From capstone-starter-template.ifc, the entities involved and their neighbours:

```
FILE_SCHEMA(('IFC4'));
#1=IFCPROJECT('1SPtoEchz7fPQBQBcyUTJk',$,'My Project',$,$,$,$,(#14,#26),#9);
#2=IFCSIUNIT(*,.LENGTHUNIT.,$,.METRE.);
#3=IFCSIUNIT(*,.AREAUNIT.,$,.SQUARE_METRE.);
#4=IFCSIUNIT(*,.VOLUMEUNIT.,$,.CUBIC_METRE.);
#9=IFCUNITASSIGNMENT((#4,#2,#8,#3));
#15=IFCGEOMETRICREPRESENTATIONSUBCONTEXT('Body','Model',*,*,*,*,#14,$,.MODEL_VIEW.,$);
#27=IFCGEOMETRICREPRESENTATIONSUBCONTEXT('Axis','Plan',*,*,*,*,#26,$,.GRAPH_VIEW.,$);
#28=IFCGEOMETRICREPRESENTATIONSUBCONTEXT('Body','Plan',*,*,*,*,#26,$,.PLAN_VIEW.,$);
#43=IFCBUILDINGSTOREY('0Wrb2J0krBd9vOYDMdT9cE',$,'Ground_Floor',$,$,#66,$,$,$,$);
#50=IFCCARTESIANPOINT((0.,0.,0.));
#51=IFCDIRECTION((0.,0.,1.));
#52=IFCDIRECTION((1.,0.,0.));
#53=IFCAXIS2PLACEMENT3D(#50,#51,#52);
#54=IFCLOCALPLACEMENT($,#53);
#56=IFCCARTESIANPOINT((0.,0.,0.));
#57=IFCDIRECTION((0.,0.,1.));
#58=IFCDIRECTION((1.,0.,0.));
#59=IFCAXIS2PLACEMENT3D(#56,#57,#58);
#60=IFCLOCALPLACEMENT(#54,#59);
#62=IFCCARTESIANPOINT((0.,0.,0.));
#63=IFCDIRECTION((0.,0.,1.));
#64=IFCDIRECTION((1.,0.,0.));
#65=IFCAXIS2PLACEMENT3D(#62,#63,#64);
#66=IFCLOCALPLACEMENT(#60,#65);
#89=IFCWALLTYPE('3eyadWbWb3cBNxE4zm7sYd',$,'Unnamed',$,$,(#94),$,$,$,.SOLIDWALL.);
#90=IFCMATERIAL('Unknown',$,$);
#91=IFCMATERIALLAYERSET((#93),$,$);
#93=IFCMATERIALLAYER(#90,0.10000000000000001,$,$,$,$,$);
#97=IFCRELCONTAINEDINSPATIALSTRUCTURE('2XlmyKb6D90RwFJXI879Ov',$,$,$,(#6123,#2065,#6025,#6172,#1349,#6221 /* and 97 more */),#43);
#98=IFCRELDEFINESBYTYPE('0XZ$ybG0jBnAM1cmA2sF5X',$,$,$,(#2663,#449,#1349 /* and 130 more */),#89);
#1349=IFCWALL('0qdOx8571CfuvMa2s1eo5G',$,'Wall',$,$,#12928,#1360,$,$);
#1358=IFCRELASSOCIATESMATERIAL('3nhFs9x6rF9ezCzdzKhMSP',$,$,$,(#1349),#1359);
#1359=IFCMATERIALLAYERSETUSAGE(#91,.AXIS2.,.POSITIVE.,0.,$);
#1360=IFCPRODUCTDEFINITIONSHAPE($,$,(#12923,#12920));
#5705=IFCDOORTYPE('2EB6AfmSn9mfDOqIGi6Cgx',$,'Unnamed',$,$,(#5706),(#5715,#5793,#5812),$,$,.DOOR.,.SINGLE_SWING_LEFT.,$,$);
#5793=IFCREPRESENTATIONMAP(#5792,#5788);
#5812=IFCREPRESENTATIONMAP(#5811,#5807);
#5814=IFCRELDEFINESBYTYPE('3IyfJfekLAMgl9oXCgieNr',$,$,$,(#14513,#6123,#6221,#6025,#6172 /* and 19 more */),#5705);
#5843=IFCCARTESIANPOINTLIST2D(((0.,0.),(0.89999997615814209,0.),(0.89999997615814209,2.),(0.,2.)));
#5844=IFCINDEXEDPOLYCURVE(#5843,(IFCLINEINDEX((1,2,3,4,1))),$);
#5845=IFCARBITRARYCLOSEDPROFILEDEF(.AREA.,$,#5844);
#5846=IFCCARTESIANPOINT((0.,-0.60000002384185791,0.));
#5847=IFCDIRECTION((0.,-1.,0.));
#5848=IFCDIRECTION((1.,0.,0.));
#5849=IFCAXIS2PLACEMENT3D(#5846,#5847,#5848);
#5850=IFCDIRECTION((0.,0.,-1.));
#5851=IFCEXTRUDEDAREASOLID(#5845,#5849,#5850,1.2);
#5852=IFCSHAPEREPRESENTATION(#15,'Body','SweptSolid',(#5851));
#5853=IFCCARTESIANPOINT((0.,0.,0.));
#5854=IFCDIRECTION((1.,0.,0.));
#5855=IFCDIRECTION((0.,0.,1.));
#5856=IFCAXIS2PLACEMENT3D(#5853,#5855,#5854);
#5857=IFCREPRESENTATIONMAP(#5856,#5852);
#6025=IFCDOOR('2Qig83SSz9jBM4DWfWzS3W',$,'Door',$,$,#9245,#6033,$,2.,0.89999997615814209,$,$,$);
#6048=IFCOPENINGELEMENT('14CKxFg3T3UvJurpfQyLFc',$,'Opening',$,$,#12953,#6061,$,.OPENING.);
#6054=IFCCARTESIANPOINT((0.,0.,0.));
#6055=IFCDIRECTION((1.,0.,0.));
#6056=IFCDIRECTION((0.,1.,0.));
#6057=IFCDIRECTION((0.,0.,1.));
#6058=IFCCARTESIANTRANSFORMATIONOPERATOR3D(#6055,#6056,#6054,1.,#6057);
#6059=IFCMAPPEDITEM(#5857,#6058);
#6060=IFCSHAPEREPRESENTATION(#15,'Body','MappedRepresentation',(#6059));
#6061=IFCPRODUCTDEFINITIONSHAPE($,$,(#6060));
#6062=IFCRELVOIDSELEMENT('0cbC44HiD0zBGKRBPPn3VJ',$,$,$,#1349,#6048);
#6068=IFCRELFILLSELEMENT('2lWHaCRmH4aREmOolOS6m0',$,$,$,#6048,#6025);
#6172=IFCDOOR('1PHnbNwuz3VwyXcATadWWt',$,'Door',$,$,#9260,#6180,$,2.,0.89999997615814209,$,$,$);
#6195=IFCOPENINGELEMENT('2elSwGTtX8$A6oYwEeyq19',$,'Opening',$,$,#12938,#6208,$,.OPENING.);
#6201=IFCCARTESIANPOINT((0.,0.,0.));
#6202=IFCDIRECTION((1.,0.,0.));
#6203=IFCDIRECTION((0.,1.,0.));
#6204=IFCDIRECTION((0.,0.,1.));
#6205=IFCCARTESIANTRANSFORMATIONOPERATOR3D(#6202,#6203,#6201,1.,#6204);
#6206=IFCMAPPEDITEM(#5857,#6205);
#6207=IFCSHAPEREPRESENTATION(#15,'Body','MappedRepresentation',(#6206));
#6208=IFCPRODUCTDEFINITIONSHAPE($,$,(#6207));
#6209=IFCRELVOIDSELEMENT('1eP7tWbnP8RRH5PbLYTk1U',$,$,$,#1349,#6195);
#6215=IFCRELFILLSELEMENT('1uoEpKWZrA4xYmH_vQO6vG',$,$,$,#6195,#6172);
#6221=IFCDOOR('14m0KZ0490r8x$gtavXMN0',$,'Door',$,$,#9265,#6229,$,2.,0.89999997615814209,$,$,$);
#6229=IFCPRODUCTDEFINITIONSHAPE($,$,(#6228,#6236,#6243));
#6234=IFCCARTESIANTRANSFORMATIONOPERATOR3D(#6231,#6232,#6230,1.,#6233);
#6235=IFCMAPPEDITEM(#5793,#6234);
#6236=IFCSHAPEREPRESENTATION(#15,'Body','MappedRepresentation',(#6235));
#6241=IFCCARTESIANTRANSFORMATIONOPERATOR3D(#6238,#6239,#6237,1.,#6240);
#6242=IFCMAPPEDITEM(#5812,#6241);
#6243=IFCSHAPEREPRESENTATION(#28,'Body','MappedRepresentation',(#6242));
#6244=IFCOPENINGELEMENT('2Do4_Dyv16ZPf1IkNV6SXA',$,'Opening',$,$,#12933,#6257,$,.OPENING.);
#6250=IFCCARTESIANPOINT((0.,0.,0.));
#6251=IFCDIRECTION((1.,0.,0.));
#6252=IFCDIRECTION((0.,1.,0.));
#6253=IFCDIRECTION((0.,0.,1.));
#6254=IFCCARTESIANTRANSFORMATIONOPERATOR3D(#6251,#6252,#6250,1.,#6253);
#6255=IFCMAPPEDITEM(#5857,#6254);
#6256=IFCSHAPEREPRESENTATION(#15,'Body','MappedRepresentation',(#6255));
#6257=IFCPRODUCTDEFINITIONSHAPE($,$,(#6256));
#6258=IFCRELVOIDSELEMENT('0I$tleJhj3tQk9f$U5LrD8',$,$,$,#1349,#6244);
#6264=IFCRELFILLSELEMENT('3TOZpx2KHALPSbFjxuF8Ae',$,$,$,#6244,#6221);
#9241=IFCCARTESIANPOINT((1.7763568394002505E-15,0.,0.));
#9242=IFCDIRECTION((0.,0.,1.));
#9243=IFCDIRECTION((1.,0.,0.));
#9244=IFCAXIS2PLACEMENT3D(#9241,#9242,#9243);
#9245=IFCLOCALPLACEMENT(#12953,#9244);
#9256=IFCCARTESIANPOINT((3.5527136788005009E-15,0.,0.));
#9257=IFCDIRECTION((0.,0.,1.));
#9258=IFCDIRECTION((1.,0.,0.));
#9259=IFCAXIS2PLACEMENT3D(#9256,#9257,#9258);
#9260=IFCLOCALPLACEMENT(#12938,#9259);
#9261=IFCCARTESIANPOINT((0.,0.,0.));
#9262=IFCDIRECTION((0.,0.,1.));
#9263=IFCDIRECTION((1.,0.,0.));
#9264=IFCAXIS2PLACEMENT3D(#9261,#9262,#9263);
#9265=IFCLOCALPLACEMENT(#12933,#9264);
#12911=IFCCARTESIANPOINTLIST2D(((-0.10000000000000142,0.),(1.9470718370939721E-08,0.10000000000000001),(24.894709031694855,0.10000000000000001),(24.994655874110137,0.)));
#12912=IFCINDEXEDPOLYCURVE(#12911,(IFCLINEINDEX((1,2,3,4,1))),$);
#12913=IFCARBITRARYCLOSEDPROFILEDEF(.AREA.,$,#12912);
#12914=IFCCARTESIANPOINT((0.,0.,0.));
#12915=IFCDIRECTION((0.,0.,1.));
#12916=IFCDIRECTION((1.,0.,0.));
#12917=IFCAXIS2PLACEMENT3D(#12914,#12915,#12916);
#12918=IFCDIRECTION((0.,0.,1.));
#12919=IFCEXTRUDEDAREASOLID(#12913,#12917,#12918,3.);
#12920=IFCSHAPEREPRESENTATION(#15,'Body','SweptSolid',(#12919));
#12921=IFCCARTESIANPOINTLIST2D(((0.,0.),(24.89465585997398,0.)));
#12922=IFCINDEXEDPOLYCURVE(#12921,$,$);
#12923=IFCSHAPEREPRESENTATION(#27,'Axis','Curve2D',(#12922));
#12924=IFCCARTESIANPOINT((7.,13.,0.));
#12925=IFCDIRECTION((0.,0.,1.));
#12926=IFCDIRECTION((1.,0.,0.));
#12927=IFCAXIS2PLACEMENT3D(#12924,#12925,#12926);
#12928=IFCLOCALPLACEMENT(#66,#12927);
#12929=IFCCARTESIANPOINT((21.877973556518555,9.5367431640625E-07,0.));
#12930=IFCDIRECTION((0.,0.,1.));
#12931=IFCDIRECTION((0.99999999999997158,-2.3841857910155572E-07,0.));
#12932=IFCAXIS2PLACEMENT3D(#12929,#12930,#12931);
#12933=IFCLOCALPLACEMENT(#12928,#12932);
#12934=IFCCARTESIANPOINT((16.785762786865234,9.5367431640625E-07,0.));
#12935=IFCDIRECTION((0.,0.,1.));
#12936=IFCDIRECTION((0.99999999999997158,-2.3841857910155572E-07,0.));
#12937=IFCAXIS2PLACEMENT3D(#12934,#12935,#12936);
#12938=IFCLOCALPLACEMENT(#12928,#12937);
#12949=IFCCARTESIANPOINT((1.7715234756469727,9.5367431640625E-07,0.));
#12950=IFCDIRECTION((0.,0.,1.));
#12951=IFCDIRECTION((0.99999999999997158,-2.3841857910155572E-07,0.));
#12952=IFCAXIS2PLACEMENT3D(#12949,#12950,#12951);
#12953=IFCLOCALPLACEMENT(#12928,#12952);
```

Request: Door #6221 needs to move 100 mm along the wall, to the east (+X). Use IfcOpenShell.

```python
import ifcopenshell
import ifcopenshell.api.geometry
import ifcopenshell.util.placement
import ifcopenshell.util.unit

model = ifcopenshell.open("capstone-starter-template.ifc")
unit_scale = ifcopenshell.util.unit.calculate_unit_scale(model)

door = model.by_guid("14m0KZ0490r8x$gtavXMN0")
opening = door.FillsVoids[0].RelatingOpeningElement
wall = opening.VoidsElements[0].RelatingBuildingElement

wall_matrix = ifcopenshell.util.placement.get_local_placement(wall.ObjectPlacement)
shift = wall_matrix[:3, 0] * 0.1 / unit_scale
before = ifcopenshell.util.placement.get_local_placement(door.ObjectPlacement)[:3, 3].copy()

# The door is placed relative to its opening, so it follows when the opening moves.
matrix = ifcopenshell.util.placement.get_local_placement(opening.ObjectPlacement)
matrix[:3, 3] += shift
ifcopenshell.api.geometry.edit_object_placement(
    model, product=opening, matrix=matrix, is_si=False, should_transform_children=True
)

after = ifcopenshell.util.placement.get_local_placement(door.ObjectPlacement)[:3, 3]
print("door moved by", (after - before).round(3) + 0.0)

model.write("capstone-starter-template_edited.ifc")
```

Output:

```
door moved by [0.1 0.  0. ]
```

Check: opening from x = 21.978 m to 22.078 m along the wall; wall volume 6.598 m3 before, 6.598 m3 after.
